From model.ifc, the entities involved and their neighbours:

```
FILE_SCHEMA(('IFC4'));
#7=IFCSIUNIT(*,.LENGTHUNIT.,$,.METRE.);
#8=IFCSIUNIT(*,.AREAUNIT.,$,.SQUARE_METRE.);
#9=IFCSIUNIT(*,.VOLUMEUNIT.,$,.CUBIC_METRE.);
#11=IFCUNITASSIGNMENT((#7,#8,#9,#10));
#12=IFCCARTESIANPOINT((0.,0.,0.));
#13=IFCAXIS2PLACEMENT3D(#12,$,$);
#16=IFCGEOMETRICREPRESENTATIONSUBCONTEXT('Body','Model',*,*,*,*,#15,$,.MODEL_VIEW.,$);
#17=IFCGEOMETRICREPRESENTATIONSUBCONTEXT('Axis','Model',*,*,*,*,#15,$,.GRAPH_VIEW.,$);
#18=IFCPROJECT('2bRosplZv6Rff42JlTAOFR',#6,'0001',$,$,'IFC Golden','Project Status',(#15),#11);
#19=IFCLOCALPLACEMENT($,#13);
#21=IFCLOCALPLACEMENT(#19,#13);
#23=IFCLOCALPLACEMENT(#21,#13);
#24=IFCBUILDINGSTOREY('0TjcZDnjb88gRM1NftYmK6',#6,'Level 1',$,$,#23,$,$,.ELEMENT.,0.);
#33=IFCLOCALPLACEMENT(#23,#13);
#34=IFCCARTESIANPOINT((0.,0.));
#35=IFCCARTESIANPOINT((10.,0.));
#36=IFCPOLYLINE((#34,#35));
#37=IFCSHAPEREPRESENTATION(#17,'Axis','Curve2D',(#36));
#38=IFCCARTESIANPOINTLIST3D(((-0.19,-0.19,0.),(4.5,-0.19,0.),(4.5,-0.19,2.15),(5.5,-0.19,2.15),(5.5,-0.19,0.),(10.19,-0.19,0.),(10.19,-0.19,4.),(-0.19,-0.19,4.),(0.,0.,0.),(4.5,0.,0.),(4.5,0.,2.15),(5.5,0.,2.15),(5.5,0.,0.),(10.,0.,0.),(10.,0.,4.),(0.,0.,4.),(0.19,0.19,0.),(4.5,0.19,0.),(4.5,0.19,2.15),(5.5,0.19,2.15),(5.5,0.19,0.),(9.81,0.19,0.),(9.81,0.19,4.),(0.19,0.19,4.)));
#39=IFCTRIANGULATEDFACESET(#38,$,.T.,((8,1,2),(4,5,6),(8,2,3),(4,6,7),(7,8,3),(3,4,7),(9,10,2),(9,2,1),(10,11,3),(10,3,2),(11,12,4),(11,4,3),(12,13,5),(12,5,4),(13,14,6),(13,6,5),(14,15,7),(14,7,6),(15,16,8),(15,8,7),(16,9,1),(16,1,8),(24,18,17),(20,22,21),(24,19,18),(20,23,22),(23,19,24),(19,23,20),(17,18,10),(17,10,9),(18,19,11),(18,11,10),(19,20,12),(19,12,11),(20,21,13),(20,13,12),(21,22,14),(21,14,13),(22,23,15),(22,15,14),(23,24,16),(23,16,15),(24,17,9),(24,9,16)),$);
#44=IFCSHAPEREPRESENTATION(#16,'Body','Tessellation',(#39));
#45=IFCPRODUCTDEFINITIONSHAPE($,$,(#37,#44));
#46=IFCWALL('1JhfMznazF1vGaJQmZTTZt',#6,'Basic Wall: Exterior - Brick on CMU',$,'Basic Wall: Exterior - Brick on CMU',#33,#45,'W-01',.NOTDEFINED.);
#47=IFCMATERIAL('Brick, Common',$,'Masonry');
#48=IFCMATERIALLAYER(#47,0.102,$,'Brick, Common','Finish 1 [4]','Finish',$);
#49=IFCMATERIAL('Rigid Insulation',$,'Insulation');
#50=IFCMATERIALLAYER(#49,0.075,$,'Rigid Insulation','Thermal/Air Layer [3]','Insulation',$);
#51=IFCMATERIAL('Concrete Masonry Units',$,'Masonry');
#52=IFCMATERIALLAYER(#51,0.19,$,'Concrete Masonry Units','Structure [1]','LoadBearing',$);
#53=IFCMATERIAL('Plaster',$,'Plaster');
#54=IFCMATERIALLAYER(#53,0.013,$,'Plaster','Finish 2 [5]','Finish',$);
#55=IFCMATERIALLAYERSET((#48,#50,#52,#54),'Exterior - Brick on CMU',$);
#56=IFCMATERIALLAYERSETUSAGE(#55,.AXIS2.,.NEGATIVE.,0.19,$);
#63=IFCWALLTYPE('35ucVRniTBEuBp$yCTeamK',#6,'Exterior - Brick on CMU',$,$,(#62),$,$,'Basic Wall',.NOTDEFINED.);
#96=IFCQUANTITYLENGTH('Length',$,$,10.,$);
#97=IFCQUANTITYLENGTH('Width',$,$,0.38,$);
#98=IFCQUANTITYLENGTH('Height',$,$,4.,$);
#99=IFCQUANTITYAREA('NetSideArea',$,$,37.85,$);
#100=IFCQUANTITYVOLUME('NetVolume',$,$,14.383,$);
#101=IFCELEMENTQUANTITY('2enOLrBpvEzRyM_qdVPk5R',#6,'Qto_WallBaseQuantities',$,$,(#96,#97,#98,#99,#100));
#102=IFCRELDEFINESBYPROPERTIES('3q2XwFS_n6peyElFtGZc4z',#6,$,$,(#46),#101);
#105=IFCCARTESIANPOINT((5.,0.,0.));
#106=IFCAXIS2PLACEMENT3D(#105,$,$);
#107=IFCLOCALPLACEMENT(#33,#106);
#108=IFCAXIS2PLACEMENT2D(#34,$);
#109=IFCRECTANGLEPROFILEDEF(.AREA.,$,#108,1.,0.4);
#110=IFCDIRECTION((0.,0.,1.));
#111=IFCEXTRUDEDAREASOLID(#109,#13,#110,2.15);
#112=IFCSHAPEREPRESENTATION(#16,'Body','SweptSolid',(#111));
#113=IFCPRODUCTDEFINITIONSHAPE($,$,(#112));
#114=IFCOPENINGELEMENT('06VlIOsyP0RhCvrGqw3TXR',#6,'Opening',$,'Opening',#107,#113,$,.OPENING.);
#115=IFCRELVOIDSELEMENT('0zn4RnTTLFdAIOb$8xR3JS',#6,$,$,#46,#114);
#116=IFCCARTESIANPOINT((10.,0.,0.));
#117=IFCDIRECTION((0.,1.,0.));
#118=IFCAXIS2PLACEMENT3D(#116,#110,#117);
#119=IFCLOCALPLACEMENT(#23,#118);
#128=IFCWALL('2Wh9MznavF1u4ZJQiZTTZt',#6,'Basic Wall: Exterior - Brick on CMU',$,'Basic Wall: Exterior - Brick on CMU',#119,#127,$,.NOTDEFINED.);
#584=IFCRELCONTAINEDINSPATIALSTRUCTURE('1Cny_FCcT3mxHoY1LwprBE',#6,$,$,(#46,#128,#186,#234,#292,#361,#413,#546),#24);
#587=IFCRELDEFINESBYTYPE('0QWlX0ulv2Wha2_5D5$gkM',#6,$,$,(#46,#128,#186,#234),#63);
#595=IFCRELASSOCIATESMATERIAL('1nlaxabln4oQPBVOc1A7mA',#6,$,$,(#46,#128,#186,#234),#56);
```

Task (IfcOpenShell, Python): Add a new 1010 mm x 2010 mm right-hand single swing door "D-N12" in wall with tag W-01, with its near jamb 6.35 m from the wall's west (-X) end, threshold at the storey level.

```python
import numpy as np
import ifcopenshell
import ifcopenshell.api.feature
import ifcopenshell.api.geometry
import ifcopenshell.api.pset
import ifcopenshell.api.root
import ifcopenshell.api.spatial
import ifcopenshell.geom
import ifcopenshell.util.element
import ifcopenshell.util.placement
import ifcopenshell.util.representation
import ifcopenshell.util.shape
import ifcopenshell.util.unit

model = ifcopenshell.open("model.ifc")
unit_scale = ifcopenshell.util.unit.calculate_unit_scale(model)
area_scale = ifcopenshell.util.unit.calculate_unit_scale(model, "AREAUNIT")
volume_scale = ifcopenshell.util.unit.calculate_unit_scale(model, "VOLUMEUNIT")
settings = ifcopenshell.geom.settings()


def volume(element):
    """Net volume in cubic metres, openings subtracted."""
    shape = ifcopenshell.geom.create_shape(settings, element)
    return ifcopenshell.util.shape.get_volume(shape.geometry)


wall = model.by_id(46)
storey = ifcopenshell.util.element.get_container(wall, ifc_class="IfcBuildingStorey")
context = ifcopenshell.util.representation.get_context(model, "Model", "Body", "MODEL_VIEW")
before = volume(wall)

width, height, from_end, sill = 1.01, 2.01, 6.35, 0.0  # metres

# The wall runs along its own X axis, and the end named is its -X end.
wall_shape = ifcopenshell.geom.create_shape(settings, wall)
x, y, z = ifcopenshell.util.shape.get_vertices(wall_shape.geometry).T
start = x.min() + from_end
face, thickness = float(y.min()), float(y.max() - y.min())
wall_matrix = ifcopenshell.util.placement.get_local_placement(wall.ObjectPlacement)
level = ifcopenshell.util.placement.get_local_placement(storey.ObjectPlacement)[2, 3]


def in_wall(x, y):
    """Placement at x, y metres in the wall's axes, at sill height."""
    matrix = wall_matrix.copy()
    matrix[:, 3] = wall_matrix @ np.array([x / unit_scale, y / unit_scale, 0.0, 1.0])
    matrix[2, 3] = level + sill / unit_scale
    return matrix


# Opening: a box that overshoots both wall faces by 50 mm.
opening = ifcopenshell.api.root.create_entity(model, ifc_class="IfcOpeningElement", predefined_type="OPENING")
box = ifcopenshell.api.geometry.add_wall_representation(
    model, context=context, length=width, height=height, thickness=thickness + 0.1
)
ifcopenshell.api.geometry.assign_representation(model, product=opening, representation=box)
ifcopenshell.api.geometry.edit_object_placement(model, product=opening, matrix=in_wall(start, face - 0.05), is_si=False)
ifcopenshell.api.feature.add_feature(model, feature=opening, element=wall)

door = ifcopenshell.api.root.create_entity(model, ifc_class="IfcDoor", name="D-N12", predefined_type="DOOR")
door.OverallWidth, door.OverallHeight = width / unit_scale, height / unit_scale
door.OperationType = "SINGLE_SWING_RIGHT"
body = ifcopenshell.api.geometry.add_door_representation(
    model,
    context=context,
    overall_width=door.OverallWidth,
    overall_height=door.OverallHeight,
    operation_type="SINGLE_SWING_RIGHT",
    lining_properties={"LiningDepth": thickness / unit_scale, "ThresholdDepth": thickness / unit_scale},
)
ifcopenshell.api.geometry.assign_representation(model, product=door, representation=body)
ifcopenshell.api.spatial.assign_container(model, products=[door], relating_structure=storey)
ifcopenshell.api.feature.add_filling(model, opening=opening, element=door)

# The lining spans the wall, so the door starts at the wall face.
ifcopenshell.api.geometry.edit_object_placement(model, product=door, matrix=in_wall(start, face), is_si=False)

after = volume(wall)

# Update the wall's stored quantities.
qto = model.by_id(ifcopenshell.util.element.get_pset(wall, "Qto_WallBaseQuantities", should_inherit=False)["id"])
ifcopenshell.api.pset.edit_qto(model, qto=qto, properties={
    "NetSideArea": after / thickness / area_scale,
    "NetVolume": after / volume_scale,
})

print(f"wall volume {before:.3f} -> {after:.3f} m3")

model.write("model_rev.ifc")
```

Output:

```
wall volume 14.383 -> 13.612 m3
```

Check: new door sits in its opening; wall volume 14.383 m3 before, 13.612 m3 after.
